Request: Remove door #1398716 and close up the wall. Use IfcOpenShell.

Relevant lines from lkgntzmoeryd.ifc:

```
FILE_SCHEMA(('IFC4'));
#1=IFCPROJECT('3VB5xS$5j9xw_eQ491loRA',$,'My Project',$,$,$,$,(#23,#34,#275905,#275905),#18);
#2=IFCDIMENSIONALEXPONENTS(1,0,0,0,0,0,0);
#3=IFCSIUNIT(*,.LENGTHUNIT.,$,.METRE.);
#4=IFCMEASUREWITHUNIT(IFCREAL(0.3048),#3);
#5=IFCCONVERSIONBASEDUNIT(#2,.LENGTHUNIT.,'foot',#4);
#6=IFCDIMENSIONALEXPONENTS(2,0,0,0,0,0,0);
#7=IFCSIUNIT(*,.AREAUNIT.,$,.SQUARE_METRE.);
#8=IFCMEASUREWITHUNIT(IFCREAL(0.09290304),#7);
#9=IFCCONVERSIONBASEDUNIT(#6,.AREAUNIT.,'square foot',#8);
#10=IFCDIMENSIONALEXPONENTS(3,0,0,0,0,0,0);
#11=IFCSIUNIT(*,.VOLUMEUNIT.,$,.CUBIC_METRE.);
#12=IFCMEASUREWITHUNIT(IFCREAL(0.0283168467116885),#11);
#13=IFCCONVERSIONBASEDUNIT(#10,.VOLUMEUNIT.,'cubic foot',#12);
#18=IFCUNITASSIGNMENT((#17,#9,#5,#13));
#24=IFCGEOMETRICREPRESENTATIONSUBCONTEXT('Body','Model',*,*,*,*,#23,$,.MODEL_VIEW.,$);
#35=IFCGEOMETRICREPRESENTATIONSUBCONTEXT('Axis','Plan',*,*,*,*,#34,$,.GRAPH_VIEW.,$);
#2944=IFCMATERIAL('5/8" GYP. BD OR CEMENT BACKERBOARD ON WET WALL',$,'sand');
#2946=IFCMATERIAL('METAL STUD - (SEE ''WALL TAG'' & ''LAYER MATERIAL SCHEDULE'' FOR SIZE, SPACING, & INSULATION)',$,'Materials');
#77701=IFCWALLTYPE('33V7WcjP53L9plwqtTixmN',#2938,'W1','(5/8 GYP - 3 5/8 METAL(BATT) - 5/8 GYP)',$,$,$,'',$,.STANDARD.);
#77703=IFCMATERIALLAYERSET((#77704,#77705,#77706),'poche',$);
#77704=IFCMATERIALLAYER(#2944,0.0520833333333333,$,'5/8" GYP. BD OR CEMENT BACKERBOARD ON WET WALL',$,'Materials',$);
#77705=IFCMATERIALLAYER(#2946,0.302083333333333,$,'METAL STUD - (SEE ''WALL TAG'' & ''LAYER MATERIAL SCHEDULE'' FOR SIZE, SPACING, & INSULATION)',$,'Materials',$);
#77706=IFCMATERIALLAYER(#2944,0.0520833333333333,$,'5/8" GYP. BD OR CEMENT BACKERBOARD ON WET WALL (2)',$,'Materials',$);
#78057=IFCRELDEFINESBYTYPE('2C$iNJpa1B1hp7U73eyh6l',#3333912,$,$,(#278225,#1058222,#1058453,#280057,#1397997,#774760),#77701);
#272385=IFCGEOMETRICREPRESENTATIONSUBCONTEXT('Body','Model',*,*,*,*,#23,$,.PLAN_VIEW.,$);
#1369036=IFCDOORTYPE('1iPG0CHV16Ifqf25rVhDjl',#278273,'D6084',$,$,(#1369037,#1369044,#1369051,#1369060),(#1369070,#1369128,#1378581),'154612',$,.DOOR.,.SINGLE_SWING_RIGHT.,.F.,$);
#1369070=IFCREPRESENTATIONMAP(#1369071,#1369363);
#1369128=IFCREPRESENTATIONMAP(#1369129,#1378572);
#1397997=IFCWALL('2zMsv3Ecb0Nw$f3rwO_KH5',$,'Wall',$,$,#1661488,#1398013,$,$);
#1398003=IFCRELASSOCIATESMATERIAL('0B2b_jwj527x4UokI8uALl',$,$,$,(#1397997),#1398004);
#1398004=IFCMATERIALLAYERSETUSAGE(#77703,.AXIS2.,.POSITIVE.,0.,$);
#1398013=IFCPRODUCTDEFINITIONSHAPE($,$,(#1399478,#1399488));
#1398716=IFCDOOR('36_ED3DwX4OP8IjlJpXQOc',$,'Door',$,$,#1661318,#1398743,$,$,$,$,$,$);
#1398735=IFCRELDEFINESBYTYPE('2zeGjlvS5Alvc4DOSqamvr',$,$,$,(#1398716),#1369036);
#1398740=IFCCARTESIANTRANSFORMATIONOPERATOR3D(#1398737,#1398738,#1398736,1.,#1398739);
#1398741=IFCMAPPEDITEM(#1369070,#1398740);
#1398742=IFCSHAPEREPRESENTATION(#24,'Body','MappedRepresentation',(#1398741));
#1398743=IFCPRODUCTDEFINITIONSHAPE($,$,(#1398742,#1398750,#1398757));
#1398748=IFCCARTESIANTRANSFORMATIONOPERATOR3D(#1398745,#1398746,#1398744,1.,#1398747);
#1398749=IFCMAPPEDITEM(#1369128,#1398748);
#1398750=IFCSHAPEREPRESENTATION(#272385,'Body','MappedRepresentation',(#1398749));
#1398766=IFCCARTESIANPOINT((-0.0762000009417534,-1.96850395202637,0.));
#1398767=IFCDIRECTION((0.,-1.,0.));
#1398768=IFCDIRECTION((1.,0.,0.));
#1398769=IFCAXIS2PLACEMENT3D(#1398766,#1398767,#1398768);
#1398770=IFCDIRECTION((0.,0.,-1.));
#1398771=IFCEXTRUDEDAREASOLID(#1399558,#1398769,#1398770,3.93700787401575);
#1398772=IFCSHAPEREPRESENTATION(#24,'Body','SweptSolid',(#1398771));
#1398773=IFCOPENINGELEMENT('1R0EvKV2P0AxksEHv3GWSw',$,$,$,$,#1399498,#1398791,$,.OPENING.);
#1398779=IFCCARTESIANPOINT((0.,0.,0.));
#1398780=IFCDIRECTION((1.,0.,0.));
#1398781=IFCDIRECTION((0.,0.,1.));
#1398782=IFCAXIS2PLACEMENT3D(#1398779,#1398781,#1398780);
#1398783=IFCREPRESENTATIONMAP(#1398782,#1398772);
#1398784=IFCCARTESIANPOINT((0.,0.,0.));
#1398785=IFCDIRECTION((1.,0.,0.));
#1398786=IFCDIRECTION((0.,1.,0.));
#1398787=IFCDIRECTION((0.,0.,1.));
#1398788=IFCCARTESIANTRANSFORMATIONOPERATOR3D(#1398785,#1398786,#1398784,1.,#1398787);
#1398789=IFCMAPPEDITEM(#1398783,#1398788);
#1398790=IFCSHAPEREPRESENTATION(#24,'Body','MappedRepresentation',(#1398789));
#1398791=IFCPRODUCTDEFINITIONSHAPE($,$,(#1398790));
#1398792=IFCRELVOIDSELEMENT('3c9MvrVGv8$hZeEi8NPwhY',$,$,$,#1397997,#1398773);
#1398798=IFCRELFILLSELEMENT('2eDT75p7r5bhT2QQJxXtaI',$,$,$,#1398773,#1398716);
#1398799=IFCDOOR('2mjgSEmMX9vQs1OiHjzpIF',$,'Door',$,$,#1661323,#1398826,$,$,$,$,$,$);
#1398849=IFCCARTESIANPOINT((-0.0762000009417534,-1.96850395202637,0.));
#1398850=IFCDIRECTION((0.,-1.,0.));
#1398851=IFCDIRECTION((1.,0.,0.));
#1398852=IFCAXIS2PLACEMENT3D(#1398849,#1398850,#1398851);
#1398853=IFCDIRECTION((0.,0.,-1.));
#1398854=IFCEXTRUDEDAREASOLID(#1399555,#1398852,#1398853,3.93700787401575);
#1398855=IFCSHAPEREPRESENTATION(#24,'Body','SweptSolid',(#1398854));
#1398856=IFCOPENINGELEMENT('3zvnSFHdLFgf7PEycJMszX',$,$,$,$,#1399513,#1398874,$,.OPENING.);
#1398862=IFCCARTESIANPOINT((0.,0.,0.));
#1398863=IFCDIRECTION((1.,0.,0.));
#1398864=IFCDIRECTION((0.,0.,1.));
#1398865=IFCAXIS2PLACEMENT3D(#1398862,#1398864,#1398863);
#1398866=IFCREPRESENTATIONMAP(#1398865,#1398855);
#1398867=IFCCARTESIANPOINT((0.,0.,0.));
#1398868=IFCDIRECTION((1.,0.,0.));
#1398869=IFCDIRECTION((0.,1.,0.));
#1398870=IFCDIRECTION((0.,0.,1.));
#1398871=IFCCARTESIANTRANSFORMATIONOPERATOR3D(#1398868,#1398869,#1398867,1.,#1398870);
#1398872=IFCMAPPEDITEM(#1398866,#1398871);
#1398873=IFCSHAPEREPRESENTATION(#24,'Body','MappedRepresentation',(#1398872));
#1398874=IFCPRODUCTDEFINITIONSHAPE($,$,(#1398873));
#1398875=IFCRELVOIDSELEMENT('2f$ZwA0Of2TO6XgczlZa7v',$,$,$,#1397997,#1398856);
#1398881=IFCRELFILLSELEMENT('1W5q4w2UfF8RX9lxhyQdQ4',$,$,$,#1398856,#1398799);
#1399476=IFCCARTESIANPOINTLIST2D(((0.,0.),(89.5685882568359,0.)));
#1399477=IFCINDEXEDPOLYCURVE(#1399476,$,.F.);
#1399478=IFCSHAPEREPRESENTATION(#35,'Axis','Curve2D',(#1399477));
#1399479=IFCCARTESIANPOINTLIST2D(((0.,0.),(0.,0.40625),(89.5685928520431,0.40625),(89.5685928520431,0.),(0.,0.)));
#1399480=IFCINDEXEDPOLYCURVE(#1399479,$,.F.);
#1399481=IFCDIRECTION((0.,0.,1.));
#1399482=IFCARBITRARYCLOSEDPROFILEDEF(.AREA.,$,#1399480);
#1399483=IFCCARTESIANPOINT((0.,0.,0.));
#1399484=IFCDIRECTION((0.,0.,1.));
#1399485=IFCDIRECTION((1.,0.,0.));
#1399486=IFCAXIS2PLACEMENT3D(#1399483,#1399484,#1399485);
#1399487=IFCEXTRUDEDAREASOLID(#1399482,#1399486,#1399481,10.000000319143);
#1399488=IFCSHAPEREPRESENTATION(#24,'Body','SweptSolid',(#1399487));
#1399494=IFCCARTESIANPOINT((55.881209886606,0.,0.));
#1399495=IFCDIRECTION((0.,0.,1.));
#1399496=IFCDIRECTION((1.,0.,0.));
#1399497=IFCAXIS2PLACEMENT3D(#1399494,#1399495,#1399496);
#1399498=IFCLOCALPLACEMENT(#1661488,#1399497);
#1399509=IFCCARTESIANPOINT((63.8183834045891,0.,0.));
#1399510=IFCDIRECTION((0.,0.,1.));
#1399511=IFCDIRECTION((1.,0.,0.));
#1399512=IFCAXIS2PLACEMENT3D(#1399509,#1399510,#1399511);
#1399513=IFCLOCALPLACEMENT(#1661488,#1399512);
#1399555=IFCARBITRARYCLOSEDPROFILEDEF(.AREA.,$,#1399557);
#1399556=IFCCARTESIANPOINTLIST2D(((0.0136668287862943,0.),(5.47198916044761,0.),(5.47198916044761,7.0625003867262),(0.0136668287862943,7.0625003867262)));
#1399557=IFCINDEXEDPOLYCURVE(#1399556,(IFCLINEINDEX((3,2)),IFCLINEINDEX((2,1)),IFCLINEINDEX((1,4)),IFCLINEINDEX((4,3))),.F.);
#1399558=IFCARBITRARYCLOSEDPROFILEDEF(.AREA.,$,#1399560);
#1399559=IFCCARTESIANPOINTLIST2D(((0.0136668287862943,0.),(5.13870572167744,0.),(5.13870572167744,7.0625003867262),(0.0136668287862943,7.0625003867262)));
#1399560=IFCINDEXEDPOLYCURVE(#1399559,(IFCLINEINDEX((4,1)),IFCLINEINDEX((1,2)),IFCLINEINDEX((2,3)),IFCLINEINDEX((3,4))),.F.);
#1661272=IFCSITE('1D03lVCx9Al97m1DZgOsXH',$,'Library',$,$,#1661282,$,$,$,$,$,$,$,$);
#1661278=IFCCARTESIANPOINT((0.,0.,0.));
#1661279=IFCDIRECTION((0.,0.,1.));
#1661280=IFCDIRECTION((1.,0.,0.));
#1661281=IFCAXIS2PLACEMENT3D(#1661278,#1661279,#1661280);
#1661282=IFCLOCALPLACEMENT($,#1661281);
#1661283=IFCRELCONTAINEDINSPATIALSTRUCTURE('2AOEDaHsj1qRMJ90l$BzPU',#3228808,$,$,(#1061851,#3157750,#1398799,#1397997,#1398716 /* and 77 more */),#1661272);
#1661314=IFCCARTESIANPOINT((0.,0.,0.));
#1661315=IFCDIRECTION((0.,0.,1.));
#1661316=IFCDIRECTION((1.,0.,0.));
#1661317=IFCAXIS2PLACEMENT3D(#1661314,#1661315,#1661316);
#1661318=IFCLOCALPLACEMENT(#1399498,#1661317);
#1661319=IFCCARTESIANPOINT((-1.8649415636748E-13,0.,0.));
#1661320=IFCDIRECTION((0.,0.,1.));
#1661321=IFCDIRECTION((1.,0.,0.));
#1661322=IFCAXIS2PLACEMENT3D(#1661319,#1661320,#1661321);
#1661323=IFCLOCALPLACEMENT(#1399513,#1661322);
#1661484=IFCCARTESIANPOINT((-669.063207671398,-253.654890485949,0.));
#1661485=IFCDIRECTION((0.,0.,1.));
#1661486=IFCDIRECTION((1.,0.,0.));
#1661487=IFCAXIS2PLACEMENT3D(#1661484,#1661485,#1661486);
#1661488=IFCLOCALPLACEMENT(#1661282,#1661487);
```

```python
import ifcopenshell
import ifcopenshell.api.feature
import ifcopenshell.api.root
import ifcopenshell.geom
import ifcopenshell.util.shape

model = ifcopenshell.open("lkgntzmoeryd.ifc")
settings = ifcopenshell.geom.settings()


def volume(element):
    """Net volume in cubic metres, openings subtracted."""
    shape = ifcopenshell.geom.create_shape(settings, element)
    return ifcopenshell.util.shape.get_volume(shape.geometry)


door = model.by_id(1398716)
opening = door.FillsVoids[0].RelatingOpeningElement
wall = opening.VoidsElements[0].RelatingBuildingElement
before = volume(wall)

ifcopenshell.api.root.remove_product(model, product=door)
ifcopenshell.api.feature.remove_feature(model, feature=opening)

after = volume(wall)

print(f"wall volume {before:.3f} -> {after:.3f} m3")

model.write("lkgntzmoeryd_edited.ifc")
```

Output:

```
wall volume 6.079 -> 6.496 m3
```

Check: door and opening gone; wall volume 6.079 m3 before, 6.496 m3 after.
